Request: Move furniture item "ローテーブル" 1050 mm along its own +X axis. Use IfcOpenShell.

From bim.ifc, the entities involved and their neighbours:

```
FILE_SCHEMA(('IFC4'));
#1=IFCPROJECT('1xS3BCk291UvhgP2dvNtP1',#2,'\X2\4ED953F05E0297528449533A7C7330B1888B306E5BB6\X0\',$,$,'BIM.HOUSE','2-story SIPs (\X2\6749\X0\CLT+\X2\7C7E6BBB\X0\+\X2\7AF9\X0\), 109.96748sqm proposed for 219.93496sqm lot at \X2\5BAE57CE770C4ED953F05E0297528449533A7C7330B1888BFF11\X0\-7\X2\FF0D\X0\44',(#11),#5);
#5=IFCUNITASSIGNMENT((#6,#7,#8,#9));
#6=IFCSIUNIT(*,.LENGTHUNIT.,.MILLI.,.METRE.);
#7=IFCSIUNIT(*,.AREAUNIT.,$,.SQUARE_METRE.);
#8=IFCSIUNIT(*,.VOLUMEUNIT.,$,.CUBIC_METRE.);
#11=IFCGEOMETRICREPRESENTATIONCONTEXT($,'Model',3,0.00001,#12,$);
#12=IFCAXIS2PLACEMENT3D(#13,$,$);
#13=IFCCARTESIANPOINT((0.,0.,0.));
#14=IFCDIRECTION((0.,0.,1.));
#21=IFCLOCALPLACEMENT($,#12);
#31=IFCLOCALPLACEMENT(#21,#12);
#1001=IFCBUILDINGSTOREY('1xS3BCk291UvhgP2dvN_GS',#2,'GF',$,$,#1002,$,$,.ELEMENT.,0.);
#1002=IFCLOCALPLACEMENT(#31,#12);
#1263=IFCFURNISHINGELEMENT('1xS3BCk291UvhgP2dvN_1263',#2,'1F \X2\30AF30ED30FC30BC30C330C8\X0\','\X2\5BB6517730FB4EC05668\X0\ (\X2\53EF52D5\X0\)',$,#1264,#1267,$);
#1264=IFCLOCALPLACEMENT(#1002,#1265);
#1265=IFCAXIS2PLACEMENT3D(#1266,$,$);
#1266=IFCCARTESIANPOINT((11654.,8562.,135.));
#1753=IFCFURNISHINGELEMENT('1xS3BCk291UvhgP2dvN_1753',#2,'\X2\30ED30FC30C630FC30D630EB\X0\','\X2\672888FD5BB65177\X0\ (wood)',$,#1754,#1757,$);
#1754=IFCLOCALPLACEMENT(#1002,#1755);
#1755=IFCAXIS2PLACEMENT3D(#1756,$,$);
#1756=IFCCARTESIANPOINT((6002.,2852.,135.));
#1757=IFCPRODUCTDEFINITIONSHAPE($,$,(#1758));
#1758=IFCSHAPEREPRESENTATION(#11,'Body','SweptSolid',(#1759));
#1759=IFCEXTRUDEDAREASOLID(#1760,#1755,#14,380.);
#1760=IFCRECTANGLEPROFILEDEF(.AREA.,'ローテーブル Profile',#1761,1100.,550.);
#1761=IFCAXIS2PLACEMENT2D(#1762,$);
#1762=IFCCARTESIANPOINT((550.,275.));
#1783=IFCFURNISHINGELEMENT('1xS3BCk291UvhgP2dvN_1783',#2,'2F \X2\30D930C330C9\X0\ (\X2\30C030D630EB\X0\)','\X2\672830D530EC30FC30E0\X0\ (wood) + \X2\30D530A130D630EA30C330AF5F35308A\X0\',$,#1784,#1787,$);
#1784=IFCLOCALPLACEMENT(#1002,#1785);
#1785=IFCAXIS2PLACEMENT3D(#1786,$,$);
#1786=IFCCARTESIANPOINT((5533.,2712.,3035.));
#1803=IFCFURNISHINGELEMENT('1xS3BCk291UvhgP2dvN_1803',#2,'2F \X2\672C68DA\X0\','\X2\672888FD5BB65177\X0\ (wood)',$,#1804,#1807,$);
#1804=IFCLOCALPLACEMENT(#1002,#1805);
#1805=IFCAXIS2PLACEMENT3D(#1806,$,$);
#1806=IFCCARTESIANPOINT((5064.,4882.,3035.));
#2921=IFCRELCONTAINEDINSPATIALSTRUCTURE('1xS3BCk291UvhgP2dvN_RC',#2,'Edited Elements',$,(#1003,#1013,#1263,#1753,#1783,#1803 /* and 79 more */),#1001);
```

```python
import ifcopenshell
import ifcopenshell.api.geometry
import ifcopenshell.util.placement
import ifcopenshell.util.unit

model = ifcopenshell.open("bim.ifc")
unit_scale = ifcopenshell.util.unit.calculate_unit_scale(model)

item = model.by_guid("1xS3BCk291UvhgP2dvN_1753")
matrix = ifcopenshell.util.placement.get_local_placement(item.ObjectPlacement)
matrix[:3, 3] += matrix[:3, 0] * 1.05 / unit_scale
ifcopenshell.api.geometry.edit_object_placement(model, product=item, matrix=matrix, is_si=False)

print(ifcopenshell.util.placement.get_local_placement(item.ObjectPlacement).round(3) + 0.0)

model.write("bim_v2.ifc")
```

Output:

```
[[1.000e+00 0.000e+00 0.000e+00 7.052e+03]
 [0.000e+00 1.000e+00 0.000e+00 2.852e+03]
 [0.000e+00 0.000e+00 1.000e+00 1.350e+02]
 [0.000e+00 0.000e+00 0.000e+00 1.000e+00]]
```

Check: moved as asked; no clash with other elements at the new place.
